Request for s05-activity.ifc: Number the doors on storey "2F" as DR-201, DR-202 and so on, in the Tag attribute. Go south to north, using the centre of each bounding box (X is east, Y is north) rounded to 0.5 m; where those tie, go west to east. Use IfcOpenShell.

First a look at what the model holds.

```python
import ifcopenshell
import ifcopenshell.util.element
import ifcopenshell.util.placement

model = ifcopenshell.open("s05-activity.ifc")
print(model.schema)
storey = next(s for s in model.by_type("IfcBuildingStorey") if s.Name == "2F")
doors = [e for e in ifcopenshell.util.element.get_decomposition(storey) if e.is_a("IfcDoor")]
for e in sorted(doors, key=lambda e: e.id()):
    origin = ifcopenshell.util.placement.get_local_placement(e.ObjectPlacement)[:3, 3]
    print(e.id(), e.Tag, e.Name, origin.round(2) + 0.0, sep=" | ")
```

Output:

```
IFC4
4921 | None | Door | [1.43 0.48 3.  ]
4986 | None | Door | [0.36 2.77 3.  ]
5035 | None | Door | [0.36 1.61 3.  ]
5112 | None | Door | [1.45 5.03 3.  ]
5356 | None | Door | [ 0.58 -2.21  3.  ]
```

```python
import ifcopenshell
import ifcopenshell.geom
import ifcopenshell.util.element
import ifcopenshell.util.shape

model = ifcopenshell.open("s05-activity.ifc")
settings = ifcopenshell.geom.settings()
settings.set("use-world-coords", True)


def centre(element):
    shape = ifcopenshell.geom.create_shape(settings, element)
    return ifcopenshell.util.shape.get_bbox_centroid(shape.geometry)


storey = next(s for s in model.by_type("IfcBuildingStorey") if s.Name == "2F")
doors = [e for e in ifcopenshell.util.element.get_decomposition(storey) if e.is_a("IfcDoor")]

# Insertion points can sit at a corner or the storey origin, so sort by the geometry (in metres).
centres = {e: centre(e) for e in doors}
doors.sort(key=lambda e: (round(centres[e][1] / 0.5), centres[e][0]))

for i, e in enumerate(doors, start=1):
    number = f"DR-2{i:02d}"
    e.Tag = number
    print(e.id(), number)

model.write("s05-activity_updated.ifc")
```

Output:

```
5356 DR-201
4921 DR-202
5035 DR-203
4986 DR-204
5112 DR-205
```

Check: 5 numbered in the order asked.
